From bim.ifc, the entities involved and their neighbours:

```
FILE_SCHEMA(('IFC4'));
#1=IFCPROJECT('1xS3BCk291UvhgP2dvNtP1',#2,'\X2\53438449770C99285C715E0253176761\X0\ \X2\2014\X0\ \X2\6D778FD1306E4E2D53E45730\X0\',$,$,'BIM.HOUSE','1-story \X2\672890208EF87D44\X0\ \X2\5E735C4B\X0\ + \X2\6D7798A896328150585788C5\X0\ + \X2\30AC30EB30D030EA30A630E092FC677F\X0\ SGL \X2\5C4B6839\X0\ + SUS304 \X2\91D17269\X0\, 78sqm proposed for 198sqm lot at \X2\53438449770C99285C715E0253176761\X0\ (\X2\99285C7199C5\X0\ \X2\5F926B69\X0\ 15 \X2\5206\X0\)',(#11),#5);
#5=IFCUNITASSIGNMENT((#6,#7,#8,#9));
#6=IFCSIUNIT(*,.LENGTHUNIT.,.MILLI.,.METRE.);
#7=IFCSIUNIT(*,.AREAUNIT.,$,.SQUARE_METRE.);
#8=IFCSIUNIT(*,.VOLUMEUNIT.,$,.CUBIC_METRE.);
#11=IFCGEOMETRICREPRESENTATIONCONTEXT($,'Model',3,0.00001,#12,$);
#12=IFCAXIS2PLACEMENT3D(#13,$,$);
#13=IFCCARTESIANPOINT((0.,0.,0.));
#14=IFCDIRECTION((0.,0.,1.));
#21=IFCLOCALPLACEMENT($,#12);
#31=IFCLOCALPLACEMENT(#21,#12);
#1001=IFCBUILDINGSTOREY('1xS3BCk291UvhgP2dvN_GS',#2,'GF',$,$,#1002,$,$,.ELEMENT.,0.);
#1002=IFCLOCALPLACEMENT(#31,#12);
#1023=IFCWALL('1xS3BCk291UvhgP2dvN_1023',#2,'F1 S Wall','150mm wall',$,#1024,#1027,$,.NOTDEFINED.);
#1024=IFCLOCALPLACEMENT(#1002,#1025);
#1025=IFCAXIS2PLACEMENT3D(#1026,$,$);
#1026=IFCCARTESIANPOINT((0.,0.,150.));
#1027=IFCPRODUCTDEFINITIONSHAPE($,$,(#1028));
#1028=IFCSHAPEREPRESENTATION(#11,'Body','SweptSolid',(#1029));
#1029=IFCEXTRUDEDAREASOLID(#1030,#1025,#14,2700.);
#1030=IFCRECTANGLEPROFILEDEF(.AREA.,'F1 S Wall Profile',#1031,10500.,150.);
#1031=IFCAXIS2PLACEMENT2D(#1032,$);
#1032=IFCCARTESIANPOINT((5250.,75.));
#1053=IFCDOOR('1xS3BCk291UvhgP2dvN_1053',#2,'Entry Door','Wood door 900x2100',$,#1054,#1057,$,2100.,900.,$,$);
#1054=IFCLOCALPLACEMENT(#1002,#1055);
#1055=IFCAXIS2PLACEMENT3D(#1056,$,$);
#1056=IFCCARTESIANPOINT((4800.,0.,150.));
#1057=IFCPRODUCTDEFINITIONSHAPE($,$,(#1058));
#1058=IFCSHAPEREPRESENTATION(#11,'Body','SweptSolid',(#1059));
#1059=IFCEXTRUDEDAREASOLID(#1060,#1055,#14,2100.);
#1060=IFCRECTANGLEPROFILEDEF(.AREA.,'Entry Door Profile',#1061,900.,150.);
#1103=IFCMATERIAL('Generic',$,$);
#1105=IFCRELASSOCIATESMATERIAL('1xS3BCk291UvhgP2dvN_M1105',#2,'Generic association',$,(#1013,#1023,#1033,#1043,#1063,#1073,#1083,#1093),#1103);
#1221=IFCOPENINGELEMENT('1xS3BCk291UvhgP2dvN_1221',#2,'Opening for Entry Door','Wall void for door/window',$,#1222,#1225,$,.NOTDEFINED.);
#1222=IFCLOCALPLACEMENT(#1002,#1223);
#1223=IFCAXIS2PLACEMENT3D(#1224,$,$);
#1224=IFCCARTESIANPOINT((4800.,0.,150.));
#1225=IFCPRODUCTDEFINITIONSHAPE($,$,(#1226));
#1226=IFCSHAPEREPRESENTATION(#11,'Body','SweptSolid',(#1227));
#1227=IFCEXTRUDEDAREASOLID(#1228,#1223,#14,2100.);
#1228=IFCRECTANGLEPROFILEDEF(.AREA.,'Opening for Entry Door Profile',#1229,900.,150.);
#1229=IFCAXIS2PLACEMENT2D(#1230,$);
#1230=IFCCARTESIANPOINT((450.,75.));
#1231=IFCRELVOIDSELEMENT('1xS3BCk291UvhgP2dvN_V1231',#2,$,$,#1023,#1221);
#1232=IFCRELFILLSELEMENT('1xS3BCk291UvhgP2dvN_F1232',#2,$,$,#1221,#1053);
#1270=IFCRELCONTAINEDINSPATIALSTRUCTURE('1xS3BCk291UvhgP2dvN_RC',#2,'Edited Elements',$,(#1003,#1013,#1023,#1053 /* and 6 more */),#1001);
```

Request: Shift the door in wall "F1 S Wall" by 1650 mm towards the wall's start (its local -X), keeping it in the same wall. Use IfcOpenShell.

```python
import ifcopenshell
import ifcopenshell.api.geometry
import ifcopenshell.util.placement

model = ifcopenshell.open("bim.ifc")

door = model.by_guid("1xS3BCk291UvhgP2dvN_1053")
opening = door.FillsVoids[0].RelatingOpeningElement
wall = opening.VoidsElements[0].RelatingBuildingElement

wall_matrix = ifcopenshell.util.placement.get_local_placement(wall.ObjectPlacement)
shift = wall_matrix[:3, 0] * -1650.0
before = ifcopenshell.util.placement.get_local_placement(door.ObjectPlacement)[:3, 3].copy()

# The door is not placed relative to its opening, so move both.
for product in (opening, door):
    matrix = ifcopenshell.util.placement.get_local_placement(product.ObjectPlacement)
    matrix[:3, 3] += shift
    ifcopenshell.api.geometry.edit_object_placement(model, product=product, matrix=matrix, is_si=False)

after = ifcopenshell.util.placement.get_local_placement(door.ObjectPlacement)[:3, 3]
print("door moved by", (after - before).round(3) + 0.0)

model.write("bim_edited.ifc")
```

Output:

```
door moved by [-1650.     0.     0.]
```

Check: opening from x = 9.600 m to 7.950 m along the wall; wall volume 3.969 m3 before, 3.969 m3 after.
